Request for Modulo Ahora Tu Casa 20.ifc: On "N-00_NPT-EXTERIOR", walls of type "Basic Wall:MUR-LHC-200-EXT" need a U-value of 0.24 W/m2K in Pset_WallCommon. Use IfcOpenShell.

First a look at what the model holds.

```python
import ifcopenshell
import ifcopenshell.util.element

model = ifcopenshell.open("Modulo Ahora Tu Casa 20.ifc")
print(model.schema)
storey = next(s for s in model.by_type("IfcBuildingStorey") if s.Name == "N-00_NPT-EXTERIOR")
walls = [e for e in ifcopenshell.util.element.get_decomposition(storey) if e.is_a("IfcWall")]
seen = {}
for e in walls:
    element_type = ifcopenshell.util.element.get_type(e)
    key = (element_type.Name if element_type != e and element_type else None, ifcopenshell.util.element.get_pset(e, "Pset_WallCommon", "ThermalTransmittance"))
    seen[key] = seen.get(key, 0) + 1
for (name, value), count in sorted(seen.items(), key=str):
    print(count, "x", name, "|", value)
```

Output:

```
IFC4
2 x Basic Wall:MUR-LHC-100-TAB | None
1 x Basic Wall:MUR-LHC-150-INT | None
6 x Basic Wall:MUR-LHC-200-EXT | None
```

```python
import ifcopenshell
import ifcopenshell.api.pset
import ifcopenshell.util.element

model = ifcopenshell.open("Modulo Ahora Tu Casa 20.ifc")

storey = next(s for s in model.by_type("IfcBuildingStorey") if s.Name == "N-00_NPT-EXTERIOR")
walls = [e for e in ifcopenshell.util.element.get_decomposition(storey) if e.is_a("IfcWall")]

count = 0
for e in walls:
    element_type = ifcopenshell.util.element.get_type(e)
    if element_type in (None, e) or element_type.Name != "Basic Wall:MUR-LHC-200-EXT":
        continue
    # add_pset returns the element's existing set when there is one.
    pset = ifcopenshell.api.pset.add_pset(model, product=e, name="Pset_WallCommon")
    ifcopenshell.api.pset.edit_pset(model, pset=pset, properties={"ThermalTransmittance": 0.24})
    count += 1

print(count, "walls updated")

model.write("Modulo Ahora Tu Casa 20_updated.ifc")
```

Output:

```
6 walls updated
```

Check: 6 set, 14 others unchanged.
